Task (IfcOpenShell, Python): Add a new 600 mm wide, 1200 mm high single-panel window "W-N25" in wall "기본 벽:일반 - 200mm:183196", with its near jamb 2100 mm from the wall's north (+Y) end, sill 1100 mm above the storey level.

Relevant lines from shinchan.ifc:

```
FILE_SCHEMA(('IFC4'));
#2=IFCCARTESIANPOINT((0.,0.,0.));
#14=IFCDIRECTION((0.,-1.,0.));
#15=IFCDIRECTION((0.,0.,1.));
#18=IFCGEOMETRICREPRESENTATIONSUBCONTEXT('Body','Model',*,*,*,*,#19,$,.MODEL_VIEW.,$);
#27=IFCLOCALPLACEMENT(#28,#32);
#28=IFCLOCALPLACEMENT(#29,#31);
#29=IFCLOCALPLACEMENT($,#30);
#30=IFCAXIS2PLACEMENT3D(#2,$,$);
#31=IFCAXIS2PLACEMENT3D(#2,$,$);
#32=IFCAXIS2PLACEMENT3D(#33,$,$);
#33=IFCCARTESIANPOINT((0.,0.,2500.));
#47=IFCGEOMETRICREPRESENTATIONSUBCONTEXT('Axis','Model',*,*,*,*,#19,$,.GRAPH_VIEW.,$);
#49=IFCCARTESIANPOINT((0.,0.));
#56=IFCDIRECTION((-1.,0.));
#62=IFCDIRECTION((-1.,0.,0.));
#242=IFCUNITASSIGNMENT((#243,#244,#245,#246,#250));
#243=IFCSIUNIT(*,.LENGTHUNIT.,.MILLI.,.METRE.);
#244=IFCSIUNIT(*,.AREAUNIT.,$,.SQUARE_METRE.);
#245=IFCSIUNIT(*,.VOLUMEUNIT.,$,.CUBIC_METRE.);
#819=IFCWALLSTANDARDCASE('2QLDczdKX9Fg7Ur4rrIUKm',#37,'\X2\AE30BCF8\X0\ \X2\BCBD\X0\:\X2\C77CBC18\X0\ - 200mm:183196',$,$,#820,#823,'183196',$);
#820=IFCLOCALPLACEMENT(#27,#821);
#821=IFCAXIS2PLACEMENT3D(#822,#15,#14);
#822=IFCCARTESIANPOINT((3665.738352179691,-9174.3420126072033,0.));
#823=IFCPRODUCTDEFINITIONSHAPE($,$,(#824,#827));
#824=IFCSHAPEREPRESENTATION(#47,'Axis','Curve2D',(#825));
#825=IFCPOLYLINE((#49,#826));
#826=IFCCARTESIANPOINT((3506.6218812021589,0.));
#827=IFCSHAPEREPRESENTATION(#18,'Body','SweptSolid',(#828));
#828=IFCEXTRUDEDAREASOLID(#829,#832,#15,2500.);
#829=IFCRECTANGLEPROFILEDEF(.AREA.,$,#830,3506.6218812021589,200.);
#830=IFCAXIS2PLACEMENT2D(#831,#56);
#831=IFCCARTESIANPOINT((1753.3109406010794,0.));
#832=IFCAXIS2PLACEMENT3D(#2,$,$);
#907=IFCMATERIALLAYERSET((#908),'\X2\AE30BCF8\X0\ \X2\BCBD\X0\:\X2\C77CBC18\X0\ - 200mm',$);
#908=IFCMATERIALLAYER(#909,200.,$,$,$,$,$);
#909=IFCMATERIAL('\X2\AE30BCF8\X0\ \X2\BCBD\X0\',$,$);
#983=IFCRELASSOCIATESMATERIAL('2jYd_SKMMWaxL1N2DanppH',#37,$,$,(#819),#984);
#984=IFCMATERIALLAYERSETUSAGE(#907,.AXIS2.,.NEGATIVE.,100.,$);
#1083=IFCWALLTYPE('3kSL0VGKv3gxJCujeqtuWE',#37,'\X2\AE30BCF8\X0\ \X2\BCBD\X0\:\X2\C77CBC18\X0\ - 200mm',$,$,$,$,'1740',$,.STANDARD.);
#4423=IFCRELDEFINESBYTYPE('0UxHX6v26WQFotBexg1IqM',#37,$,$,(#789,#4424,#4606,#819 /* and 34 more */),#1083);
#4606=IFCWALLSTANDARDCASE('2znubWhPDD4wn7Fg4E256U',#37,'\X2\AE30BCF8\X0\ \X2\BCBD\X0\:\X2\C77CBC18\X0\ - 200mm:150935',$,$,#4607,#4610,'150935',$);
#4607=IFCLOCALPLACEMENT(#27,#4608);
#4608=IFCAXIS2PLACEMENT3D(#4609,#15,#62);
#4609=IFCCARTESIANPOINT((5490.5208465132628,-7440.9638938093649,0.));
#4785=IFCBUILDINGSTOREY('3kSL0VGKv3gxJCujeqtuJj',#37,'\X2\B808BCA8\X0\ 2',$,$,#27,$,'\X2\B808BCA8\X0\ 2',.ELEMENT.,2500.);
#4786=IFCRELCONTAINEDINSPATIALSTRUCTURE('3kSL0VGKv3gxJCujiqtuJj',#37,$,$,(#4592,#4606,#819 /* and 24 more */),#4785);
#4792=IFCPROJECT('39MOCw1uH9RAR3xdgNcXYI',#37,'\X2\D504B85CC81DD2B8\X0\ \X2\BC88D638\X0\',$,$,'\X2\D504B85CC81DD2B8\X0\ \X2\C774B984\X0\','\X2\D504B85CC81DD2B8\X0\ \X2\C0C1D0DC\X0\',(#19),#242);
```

```python
import numpy as np
import ifcopenshell
import ifcopenshell.api.feature
import ifcopenshell.api.geometry
import ifcopenshell.api.root
import ifcopenshell.api.spatial
import ifcopenshell.geom
import ifcopenshell.util.element
import ifcopenshell.util.placement
import ifcopenshell.util.representation
import ifcopenshell.util.shape
import ifcopenshell.util.unit

model = ifcopenshell.open("shinchan.ifc")
unit_scale = ifcopenshell.util.unit.calculate_unit_scale(model)
settings = ifcopenshell.geom.settings()


def volume(element):
    """Net volume in cubic metres, openings subtracted."""
    shape = ifcopenshell.geom.create_shape(settings, element)
    return ifcopenshell.util.shape.get_volume(shape.geometry)


wall = model.by_guid("2QLDczdKX9Fg7Ur4rrIUKm")
storey = ifcopenshell.util.element.get_container(wall, ifc_class="IfcBuildingStorey")
context = ifcopenshell.util.representation.get_context(model, "Model", "Body", "MODEL_VIEW")
before = volume(wall)

width, height, from_end, sill = 0.6, 1.2, 2.1, 1.1  # metres

# The wall runs along its own X axis, and the end named is its -X end.
wall_shape = ifcopenshell.geom.create_shape(settings, wall)
x, y, z = ifcopenshell.util.shape.get_vertices(wall_shape.geometry).T
start = x.min() + from_end
face, thickness = float(y.min()), float(y.max() - y.min())
wall_matrix = ifcopenshell.util.placement.get_local_placement(wall.ObjectPlacement)
level = ifcopenshell.util.placement.get_local_placement(storey.ObjectPlacement)[2, 3]


def in_wall(x, y):
    """Placement at x, y metres in the wall's axes, at sill height."""
    matrix = wall_matrix.copy()
    matrix[:, 3] = wall_matrix @ np.array([x / unit_scale, y / unit_scale, 0.0, 1.0])
    matrix[2, 3] = level + sill / unit_scale
    return matrix


# Opening: a box that overshoots both wall faces by 50 mm.
opening = ifcopenshell.api.root.create_entity(model, ifc_class="IfcOpeningElement", predefined_type="OPENING")
box = ifcopenshell.api.geometry.add_wall_representation(
    model, context=context, length=width, height=height, thickness=thickness + 0.1
)
ifcopenshell.api.geometry.assign_representation(model, product=opening, representation=box)
ifcopenshell.api.geometry.edit_object_placement(model, product=opening, matrix=in_wall(start, face - 0.05), is_si=False)
ifcopenshell.api.feature.add_feature(model, feature=opening, element=wall)

window = ifcopenshell.api.root.create_entity(model, ifc_class="IfcWindow", name="W-N25", predefined_type="WINDOW")
window.OverallWidth, window.OverallHeight = width / unit_scale, height / unit_scale
window.PartitioningType = "SINGLE_PANEL"
body = ifcopenshell.api.geometry.add_window_representation(
    model,
    context=context,
    overall_width=window.OverallWidth,
    overall_height=window.OverallHeight,
    partition_type="SINGLE_PANEL",
)
ifcopenshell.api.geometry.assign_representation(model, product=window, representation=body)
ifcopenshell.api.spatial.assign_container(model, products=[window], relating_structure=storey)
ifcopenshell.api.feature.add_filling(model, opening=opening, element=window)

# Centre the window in the wall's thickness.
ifcopenshell.api.geometry.edit_object_placement(model, product=window, matrix=in_wall(start, face), is_si=False)
window_shape = ifcopenshell.geom.create_shape(settings, window)
depth = ifcopenshell.util.shape.get_vertices(window_shape.geometry)[:, 1]
offset = face + thickness / 2 - (depth.min() + depth.max()) / 2
ifcopenshell.api.geometry.edit_object_placement(model, product=window, matrix=in_wall(start, offset), is_si=False)

after = volume(wall)

print(f"wall volume {before:.3f} -> {after:.3f} m3")

model.write("shinchan_rev.ifc")
```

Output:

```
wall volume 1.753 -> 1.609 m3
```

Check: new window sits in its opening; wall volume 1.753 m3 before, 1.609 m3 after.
